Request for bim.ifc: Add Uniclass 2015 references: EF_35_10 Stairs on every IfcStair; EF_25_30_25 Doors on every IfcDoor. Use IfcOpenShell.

First a look at what the model holds.

```python
import ifcopenshell

model = ifcopenshell.open("bim.ifc")
print(model.schema)
print("classifications:", [c.Name for c in model.by_type("IfcClassification")])
for ifc_class in ("IfcDoor", "IfcRoof", "IfcStair", "IfcWall", "IfcWindow"):
    print(ifc_class, len(model.by_type(ifc_class)))
```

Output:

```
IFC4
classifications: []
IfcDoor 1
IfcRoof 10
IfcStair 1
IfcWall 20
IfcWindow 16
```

```python
import ifcopenshell
import ifcopenshell.api.classification

model = ifcopenshell.open("bim.ifc")

system = ifcopenshell.api.classification.add_classification(model, classification="Uniclass 2015")

codes = {
    "IfcStair": ("EF_35_10", "Stairs"),
    "IfcDoor": ("EF_25_30_25", "Doors"),
}
for ifc_class, (code, name) in codes.items():
    products = model.by_type(ifc_class)
    ifcopenshell.api.classification.add_reference(
        model, products=products, classification=system, identification=code, name=name
    )
    print(code, len(products))

model.write("bim_v2.ifc")
```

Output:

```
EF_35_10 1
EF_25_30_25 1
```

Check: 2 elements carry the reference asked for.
